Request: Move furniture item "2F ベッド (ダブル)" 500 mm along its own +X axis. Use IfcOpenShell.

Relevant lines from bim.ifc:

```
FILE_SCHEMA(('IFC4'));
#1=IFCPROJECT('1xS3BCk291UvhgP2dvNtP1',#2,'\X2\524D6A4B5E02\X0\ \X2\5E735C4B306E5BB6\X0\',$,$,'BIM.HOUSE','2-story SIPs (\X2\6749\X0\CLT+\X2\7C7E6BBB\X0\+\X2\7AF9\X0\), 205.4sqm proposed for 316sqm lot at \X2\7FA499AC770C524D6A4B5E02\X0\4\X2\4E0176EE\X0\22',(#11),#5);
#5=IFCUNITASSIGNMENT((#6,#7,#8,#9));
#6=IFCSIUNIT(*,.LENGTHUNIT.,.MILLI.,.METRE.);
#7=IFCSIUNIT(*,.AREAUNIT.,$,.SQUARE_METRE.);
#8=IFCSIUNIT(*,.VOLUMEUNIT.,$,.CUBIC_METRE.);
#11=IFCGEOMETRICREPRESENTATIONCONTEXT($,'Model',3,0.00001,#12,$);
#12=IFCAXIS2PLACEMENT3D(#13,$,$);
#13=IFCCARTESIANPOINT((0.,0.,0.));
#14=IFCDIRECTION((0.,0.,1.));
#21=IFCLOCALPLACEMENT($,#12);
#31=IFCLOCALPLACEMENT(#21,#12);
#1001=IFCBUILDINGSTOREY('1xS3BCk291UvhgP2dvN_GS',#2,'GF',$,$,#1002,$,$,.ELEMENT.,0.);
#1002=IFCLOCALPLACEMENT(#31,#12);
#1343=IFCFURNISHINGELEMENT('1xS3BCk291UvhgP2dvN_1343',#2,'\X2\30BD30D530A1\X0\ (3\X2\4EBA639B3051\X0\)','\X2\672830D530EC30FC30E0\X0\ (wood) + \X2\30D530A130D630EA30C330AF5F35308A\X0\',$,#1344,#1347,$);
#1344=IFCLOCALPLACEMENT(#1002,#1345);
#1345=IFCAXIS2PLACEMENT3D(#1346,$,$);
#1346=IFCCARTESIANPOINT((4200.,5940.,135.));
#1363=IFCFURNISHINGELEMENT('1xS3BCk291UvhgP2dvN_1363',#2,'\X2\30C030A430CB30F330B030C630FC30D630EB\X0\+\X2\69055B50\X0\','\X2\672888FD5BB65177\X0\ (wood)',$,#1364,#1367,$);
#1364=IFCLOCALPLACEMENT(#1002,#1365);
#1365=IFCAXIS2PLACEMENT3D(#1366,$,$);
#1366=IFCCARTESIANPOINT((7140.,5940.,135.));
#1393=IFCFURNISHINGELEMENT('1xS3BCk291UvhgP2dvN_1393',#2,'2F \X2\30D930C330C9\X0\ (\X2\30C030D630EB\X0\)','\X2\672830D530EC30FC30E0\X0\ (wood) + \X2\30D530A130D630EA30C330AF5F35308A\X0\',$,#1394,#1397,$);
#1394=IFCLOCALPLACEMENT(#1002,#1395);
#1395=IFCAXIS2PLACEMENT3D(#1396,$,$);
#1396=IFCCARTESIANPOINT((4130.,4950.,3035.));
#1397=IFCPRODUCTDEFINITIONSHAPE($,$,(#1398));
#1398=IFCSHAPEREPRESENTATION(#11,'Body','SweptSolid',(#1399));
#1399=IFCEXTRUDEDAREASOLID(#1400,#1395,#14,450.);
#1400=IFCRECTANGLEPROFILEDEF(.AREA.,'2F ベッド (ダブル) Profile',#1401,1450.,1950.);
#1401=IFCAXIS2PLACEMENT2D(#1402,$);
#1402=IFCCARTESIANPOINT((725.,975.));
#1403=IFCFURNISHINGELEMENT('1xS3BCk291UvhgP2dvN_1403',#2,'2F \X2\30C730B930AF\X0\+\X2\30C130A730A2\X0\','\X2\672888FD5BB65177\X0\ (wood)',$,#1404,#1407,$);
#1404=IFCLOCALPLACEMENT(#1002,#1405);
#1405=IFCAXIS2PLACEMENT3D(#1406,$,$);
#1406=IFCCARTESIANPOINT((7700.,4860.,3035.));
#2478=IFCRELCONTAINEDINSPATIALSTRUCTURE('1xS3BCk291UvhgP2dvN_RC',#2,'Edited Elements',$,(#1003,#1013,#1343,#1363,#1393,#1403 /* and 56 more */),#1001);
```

```python
import ifcopenshell
import ifcopenshell.api.geometry
import ifcopenshell.util.placement

model = ifcopenshell.open("bim.ifc")

item = model.by_id(1393)
matrix = ifcopenshell.util.placement.get_local_placement(item.ObjectPlacement)
matrix[:3, 3] += matrix[:3, 0] * 500.0
ifcopenshell.api.geometry.edit_object_placement(model, product=item, matrix=matrix, is_si=False)

print(ifcopenshell.util.placement.get_local_placement(item.ObjectPlacement).round(3) + 0.0)

model.write("bim_rev.ifc")
```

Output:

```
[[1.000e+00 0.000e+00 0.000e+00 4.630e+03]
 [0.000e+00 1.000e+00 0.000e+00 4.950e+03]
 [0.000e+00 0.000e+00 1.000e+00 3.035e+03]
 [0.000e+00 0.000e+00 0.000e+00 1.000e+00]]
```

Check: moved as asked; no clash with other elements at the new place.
